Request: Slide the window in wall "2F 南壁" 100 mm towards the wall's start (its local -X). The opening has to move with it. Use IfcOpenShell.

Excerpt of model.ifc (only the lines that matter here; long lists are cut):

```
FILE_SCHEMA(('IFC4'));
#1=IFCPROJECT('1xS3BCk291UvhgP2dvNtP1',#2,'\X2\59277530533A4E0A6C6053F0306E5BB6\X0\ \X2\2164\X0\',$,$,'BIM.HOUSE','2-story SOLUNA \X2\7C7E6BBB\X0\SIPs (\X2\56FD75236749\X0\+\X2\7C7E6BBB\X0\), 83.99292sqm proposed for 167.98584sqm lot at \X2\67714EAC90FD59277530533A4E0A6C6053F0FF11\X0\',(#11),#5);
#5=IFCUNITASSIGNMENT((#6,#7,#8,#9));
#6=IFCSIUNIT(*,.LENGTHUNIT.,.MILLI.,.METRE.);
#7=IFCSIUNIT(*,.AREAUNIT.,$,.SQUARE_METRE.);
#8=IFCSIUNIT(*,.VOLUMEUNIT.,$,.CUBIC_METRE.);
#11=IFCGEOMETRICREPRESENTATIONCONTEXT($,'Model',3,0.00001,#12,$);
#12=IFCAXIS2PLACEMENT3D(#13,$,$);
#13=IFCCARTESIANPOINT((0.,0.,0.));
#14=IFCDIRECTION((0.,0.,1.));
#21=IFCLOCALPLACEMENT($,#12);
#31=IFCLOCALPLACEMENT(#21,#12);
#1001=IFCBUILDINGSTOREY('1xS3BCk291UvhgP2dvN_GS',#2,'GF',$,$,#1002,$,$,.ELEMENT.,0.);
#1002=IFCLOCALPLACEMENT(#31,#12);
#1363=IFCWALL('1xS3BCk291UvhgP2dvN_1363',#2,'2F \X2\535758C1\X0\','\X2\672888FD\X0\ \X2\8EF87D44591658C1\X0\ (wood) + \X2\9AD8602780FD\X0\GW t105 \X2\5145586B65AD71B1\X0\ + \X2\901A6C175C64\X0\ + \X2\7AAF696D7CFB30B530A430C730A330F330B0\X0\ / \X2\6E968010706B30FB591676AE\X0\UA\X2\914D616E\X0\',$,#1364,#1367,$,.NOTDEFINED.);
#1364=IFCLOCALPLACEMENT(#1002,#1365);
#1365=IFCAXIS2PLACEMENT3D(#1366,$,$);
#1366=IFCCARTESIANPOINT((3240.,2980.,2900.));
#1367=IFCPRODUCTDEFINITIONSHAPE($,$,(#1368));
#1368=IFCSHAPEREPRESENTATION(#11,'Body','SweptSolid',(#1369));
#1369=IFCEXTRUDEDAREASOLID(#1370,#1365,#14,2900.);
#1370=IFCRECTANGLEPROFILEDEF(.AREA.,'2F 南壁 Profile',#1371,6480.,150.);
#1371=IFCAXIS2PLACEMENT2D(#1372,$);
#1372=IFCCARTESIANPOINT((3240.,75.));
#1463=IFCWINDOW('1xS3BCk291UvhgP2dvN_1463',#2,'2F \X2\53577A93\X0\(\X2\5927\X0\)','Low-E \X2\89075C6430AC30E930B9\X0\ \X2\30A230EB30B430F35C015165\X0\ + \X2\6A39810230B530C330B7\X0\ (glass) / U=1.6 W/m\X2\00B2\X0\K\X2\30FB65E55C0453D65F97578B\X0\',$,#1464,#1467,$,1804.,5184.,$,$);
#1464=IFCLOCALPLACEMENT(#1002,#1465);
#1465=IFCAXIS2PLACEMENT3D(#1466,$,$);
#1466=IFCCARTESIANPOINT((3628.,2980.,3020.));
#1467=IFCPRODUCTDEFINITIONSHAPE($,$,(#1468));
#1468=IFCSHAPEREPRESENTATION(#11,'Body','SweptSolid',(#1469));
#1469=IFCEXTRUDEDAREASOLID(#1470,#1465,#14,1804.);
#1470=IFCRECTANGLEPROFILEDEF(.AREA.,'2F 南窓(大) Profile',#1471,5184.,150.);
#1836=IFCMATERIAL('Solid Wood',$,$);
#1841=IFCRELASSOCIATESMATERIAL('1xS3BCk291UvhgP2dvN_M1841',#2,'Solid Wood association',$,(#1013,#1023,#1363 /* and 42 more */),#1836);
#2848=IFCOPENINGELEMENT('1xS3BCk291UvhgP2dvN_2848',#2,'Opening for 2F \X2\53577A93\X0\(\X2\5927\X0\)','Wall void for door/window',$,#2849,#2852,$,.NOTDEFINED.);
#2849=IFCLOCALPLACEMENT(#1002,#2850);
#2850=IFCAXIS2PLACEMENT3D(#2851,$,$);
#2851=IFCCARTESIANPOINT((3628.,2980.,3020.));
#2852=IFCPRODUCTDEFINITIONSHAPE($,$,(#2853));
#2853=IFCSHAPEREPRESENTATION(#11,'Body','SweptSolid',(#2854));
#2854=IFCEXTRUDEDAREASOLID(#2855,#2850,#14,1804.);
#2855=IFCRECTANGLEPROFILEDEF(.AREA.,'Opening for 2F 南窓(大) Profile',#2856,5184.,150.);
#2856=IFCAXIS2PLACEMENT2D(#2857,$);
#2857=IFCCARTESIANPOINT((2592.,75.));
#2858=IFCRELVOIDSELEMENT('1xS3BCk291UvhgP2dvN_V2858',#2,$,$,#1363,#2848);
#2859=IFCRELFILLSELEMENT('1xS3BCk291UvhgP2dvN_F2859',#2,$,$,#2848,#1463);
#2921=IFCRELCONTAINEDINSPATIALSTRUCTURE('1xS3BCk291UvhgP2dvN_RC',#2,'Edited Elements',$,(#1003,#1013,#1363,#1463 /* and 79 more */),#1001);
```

```python
import ifcopenshell
import ifcopenshell.api.geometry
import ifcopenshell.util.placement
import ifcopenshell.util.unit

model = ifcopenshell.open("model.ifc")
unit_scale = ifcopenshell.util.unit.calculate_unit_scale(model)

window = model.by_guid("1xS3BCk291UvhgP2dvN_1463")
opening = window.FillsVoids[0].RelatingOpeningElement
wall = opening.VoidsElements[0].RelatingBuildingElement

wall_matrix = ifcopenshell.util.placement.get_local_placement(wall.ObjectPlacement)
shift = wall_matrix[:3, 0] * -0.1 / unit_scale
before = ifcopenshell.util.placement.get_local_placement(window.ObjectPlacement)[:3, 3].copy()

# The window is not placed relative to its opening, so move both.
for product in (opening, window):
    matrix = ifcopenshell.util.placement.get_local_placement(product.ObjectPlacement)
    matrix[:3, 3] += shift
    ifcopenshell.api.geometry.edit_object_placement(model, product=product, matrix=matrix, is_si=False)

after = ifcopenshell.util.placement.get_local_placement(window.ObjectPlacement)[:3, 3]
print("window moved by", (after - before).round(3) + 0.0)

model.write("model_v2.ifc")
```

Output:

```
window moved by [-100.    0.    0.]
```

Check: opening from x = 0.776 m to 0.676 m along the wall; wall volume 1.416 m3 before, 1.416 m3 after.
